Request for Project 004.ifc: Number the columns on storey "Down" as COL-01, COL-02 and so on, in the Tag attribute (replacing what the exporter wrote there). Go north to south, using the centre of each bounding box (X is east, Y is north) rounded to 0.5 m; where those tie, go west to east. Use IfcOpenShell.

First a look at what the model holds.

```python
import ifcopenshell
import ifcopenshell.util.element
import ifcopenshell.util.placement

model = ifcopenshell.open("Project 004.ifc")
print(model.schema)
storey = next(s for s in model.by_type("IfcBuildingStorey") if s.Name == "Down")
columns = [e for e in ifcopenshell.util.element.get_decomposition(storey) if e.is_a("IfcColumn")]
for e in sorted(columns, key=lambda e: e.id()):
    origin = ifcopenshell.util.placement.get_local_placement(e.ObjectPlacement)[:3, 3]
    print(e.id(), e.Tag, e.Name, origin.round(2) + 0.0, sep=" | ")
```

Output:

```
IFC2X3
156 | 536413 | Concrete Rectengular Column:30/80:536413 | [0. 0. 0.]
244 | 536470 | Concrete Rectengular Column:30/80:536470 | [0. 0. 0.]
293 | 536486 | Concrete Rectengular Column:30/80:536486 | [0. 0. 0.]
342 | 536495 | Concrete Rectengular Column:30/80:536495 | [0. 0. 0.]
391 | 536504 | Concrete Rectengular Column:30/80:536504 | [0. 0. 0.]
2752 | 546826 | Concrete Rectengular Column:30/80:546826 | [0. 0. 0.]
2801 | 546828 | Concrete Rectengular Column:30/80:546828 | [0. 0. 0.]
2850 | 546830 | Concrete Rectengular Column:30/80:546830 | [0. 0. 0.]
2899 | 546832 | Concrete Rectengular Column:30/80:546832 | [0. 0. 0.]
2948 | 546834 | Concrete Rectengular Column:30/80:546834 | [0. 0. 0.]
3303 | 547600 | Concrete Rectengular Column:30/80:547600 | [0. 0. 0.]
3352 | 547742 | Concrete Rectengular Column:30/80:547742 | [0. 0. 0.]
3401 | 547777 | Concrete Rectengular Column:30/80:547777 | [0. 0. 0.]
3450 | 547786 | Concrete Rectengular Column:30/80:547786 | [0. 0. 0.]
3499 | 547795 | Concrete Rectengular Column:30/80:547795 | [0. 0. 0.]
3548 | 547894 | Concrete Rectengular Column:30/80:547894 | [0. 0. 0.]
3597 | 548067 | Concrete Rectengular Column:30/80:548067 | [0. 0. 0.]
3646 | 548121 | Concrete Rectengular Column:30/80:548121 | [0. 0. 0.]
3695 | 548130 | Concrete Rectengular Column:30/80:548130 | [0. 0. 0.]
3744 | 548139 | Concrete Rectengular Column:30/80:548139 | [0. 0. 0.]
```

```python
import ifcopenshell
import ifcopenshell.geom
import ifcopenshell.util.element
import ifcopenshell.util.shape

model = ifcopenshell.open("Project 004.ifc")
settings = ifcopenshell.geom.settings()
settings.set("use-world-coords", True)


def centre(element):
    shape = ifcopenshell.geom.create_shape(settings, element)
    return ifcopenshell.util.shape.get_bbox_centroid(shape.geometry)


storey = next(s for s in model.by_type("IfcBuildingStorey") if s.Name == "Down")
columns = [e for e in ifcopenshell.util.element.get_decomposition(storey) if e.is_a("IfcColumn")]

# Insertion points can sit at a corner or the storey origin, so sort by the geometry (in metres).
centres = {e: centre(e) for e in columns}
columns.sort(key=lambda e: (-round(centres[e][1] / 0.5), centres[e][0]))

for i, e in enumerate(columns, start=1):
    number = f"COL-{i:02d}"
    e.Tag = number
    print(e.id(), number)

model.write("Project 004_updated.ifc")
```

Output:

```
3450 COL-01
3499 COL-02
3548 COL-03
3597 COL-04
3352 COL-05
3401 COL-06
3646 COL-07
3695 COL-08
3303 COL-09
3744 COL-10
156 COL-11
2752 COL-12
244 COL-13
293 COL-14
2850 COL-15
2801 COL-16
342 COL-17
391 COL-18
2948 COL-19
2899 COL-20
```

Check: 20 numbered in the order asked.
